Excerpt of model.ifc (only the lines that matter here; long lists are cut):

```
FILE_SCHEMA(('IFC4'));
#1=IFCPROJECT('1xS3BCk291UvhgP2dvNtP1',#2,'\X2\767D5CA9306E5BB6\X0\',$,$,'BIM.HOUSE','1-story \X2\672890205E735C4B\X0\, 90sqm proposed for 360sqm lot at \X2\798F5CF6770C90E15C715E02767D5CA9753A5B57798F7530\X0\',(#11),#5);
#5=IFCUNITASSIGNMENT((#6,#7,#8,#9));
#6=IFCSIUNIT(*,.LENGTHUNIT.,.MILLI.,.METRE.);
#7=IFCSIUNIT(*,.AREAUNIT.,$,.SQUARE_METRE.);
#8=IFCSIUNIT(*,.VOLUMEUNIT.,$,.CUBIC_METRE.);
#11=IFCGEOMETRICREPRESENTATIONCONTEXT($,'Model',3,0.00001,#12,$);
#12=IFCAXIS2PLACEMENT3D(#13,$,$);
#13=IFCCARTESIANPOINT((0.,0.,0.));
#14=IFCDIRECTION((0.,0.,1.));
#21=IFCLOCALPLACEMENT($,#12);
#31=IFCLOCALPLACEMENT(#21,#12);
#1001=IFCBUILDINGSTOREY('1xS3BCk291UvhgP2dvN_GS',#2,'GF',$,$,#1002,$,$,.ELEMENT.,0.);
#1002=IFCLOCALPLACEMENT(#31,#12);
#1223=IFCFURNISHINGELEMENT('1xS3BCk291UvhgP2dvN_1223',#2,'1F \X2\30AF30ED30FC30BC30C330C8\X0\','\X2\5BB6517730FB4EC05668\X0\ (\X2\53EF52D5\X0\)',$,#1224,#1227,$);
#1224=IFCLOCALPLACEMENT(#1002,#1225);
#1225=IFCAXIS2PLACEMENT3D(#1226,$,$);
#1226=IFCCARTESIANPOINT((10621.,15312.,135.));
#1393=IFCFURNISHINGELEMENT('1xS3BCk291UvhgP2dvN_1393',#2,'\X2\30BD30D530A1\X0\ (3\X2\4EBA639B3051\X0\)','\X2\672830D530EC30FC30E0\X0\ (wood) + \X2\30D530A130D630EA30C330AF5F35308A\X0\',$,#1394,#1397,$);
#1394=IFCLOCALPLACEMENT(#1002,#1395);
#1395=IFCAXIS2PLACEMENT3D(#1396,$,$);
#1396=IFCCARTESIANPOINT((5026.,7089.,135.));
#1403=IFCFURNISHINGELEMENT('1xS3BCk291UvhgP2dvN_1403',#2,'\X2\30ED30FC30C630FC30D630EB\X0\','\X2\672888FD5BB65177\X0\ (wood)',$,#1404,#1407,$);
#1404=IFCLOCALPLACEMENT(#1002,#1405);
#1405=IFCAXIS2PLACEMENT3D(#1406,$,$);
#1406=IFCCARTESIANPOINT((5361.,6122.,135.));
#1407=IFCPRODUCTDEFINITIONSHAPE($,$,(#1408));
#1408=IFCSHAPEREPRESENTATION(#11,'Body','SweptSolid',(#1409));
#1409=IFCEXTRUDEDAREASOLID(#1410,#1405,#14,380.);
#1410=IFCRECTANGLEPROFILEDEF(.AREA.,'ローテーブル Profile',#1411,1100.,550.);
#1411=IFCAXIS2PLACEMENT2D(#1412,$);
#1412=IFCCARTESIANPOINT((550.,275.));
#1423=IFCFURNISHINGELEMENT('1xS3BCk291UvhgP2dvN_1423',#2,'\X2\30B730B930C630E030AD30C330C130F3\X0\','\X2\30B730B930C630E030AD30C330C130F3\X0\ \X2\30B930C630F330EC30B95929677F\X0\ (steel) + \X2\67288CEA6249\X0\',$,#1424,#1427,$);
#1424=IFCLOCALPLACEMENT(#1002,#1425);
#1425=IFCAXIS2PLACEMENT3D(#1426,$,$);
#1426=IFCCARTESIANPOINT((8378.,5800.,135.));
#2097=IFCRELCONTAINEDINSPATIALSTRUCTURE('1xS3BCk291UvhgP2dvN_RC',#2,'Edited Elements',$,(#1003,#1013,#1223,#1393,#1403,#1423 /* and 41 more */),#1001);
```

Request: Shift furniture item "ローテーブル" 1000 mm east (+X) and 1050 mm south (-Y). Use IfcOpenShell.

```python
import ifcopenshell
import ifcopenshell.api.geometry
import ifcopenshell.util.placement
import ifcopenshell.util.unit

model = ifcopenshell.open("model.ifc")
unit_scale = ifcopenshell.util.unit.calculate_unit_scale(model)

item = model.by_id(1403)
matrix = ifcopenshell.util.placement.get_local_placement(item.ObjectPlacement)
matrix[0, 3] += 1 / unit_scale
matrix[1, 3] -= 1.05 / unit_scale
ifcopenshell.api.geometry.edit_object_placement(model, product=item, matrix=matrix, is_si=False)

print(ifcopenshell.util.placement.get_local_placement(item.ObjectPlacement).round(3) + 0.0)

model.write("model_v2.ifc")
```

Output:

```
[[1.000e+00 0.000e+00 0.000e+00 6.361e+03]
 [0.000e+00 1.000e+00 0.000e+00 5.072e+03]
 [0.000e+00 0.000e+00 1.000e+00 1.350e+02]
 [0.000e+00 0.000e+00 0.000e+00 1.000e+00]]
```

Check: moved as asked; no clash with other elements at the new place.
